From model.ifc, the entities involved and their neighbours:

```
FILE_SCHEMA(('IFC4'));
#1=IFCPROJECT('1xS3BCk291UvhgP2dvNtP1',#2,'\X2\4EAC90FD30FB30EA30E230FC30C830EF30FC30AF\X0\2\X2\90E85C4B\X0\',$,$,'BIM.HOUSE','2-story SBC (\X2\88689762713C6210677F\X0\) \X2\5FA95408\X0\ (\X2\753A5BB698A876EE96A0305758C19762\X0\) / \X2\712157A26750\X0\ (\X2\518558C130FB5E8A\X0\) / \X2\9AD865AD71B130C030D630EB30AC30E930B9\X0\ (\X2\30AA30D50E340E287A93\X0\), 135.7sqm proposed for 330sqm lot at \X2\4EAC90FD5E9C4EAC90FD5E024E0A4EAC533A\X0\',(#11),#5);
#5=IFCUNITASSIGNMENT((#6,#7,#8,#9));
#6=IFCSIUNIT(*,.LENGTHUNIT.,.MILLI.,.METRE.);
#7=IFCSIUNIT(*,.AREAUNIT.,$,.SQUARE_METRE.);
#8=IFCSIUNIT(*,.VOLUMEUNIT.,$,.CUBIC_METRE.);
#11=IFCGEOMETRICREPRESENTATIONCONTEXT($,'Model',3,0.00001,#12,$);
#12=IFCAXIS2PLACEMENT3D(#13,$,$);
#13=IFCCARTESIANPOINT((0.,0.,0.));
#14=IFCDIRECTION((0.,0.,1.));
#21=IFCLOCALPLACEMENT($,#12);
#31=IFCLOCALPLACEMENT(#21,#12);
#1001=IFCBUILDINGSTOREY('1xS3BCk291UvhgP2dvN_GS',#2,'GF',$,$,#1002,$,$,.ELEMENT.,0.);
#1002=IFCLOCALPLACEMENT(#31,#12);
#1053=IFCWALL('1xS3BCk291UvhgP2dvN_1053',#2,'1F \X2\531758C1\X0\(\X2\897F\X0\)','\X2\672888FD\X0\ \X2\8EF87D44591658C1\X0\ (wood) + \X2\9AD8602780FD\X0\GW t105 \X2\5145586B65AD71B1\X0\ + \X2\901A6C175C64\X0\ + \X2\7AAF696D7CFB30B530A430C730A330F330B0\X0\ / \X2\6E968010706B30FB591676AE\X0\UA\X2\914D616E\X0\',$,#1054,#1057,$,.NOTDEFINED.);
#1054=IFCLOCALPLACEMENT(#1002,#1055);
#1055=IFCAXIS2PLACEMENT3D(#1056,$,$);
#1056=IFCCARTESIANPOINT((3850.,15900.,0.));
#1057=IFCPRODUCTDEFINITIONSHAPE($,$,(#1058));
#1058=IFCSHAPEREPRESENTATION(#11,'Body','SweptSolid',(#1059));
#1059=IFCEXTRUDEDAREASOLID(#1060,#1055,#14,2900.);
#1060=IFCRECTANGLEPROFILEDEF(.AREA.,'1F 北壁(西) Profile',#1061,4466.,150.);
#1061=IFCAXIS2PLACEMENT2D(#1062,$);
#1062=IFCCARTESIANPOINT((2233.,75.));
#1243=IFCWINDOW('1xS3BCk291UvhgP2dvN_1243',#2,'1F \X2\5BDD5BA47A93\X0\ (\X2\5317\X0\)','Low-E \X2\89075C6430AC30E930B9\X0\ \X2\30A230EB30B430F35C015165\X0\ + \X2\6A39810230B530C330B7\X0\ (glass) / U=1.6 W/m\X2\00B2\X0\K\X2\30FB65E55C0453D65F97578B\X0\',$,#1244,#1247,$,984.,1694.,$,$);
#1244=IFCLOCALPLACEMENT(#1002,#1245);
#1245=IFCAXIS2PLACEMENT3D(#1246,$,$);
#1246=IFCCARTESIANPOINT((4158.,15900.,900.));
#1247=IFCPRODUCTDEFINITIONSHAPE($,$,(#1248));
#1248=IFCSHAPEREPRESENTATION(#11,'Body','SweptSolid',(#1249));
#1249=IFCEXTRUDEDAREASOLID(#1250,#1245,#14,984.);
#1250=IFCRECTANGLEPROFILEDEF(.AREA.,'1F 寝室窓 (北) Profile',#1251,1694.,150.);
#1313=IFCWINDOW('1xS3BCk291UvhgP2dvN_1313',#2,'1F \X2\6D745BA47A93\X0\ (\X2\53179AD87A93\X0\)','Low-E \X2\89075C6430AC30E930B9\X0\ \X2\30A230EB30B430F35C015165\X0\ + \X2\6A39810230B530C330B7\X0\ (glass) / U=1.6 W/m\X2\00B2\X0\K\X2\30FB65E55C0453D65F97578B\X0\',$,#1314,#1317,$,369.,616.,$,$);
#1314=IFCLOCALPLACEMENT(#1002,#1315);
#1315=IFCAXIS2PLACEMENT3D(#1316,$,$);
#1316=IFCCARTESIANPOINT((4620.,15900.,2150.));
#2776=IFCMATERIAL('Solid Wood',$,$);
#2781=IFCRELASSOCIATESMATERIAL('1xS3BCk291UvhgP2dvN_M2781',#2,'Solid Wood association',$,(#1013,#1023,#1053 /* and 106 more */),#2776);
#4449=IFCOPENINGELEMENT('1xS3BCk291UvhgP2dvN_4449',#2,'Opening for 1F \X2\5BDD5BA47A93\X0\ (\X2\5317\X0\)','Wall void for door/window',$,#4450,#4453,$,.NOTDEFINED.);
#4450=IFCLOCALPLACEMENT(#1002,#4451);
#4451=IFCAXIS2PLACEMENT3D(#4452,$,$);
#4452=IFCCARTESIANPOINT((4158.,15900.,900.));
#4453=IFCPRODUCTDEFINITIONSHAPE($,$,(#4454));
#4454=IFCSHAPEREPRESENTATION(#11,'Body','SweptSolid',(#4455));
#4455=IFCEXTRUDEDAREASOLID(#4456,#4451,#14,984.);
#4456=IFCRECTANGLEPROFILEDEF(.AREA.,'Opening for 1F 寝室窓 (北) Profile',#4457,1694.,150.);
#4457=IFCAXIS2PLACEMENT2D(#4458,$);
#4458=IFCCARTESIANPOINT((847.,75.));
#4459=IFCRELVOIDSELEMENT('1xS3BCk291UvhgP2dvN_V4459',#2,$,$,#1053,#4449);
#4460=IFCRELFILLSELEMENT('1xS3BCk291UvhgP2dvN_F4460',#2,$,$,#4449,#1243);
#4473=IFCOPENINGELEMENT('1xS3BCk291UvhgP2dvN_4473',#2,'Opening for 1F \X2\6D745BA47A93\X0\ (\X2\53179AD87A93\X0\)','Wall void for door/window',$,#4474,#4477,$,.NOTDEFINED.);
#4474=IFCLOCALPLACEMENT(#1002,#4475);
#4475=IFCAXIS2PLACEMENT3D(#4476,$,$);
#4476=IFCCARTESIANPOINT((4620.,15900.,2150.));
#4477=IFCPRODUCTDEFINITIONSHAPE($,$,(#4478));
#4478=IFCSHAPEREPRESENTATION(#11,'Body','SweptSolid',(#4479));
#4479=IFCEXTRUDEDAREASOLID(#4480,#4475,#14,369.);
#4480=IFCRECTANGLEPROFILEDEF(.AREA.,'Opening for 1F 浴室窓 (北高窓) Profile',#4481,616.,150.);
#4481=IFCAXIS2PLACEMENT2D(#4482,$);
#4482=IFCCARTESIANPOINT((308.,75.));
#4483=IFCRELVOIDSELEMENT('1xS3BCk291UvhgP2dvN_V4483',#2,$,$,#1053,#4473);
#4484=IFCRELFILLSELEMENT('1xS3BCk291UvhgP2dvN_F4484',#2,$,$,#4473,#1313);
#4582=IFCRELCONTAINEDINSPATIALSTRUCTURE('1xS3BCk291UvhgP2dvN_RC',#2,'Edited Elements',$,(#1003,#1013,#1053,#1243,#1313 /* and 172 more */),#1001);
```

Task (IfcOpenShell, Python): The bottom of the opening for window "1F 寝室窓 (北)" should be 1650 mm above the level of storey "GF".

```python
import numpy as np
import ifcopenshell
import ifcopenshell.api.geometry
import ifcopenshell.geom
import ifcopenshell.util.element
import ifcopenshell.util.placement
import ifcopenshell.util.shape
import ifcopenshell.util.unit

model = ifcopenshell.open("model.ifc")
unit_scale = ifcopenshell.util.unit.calculate_unit_scale(model)

window = model.by_guid("1xS3BCk291UvhgP2dvN_1243")
opening = window.FillsVoids[0].RelatingOpeningElement
storey = ifcopenshell.util.element.get_container(window, ifc_class="IfcBuildingStorey")
level = ifcopenshell.util.placement.get_local_placement(storey.ObjectPlacement)[2, 3]

# The opening's origin need not be at the sill, so measure its lowest point.
shape = ifcopenshell.geom.create_shape(ifcopenshell.geom.settings(), opening)
bottom = ifcopenshell.util.shape.get_shape_bottom_elevation(shape, shape.geometry) / unit_scale
dz = level + 1.65 / unit_scale - bottom

shift = np.array([0.0, 0.0, dz])
# The window is not placed relative to its opening, so move both.
for product in (opening, window):
    matrix = ifcopenshell.util.placement.get_local_placement(product.ObjectPlacement)
    matrix[:3, 3] += shift
    ifcopenshell.api.geometry.edit_object_placement(model, product=product, matrix=matrix, is_si=False)

print(f"moved by {dz * unit_scale:+.3f} m")

model.write("model_rev.ifc")
```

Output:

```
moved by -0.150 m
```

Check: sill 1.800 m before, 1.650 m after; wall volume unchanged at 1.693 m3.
